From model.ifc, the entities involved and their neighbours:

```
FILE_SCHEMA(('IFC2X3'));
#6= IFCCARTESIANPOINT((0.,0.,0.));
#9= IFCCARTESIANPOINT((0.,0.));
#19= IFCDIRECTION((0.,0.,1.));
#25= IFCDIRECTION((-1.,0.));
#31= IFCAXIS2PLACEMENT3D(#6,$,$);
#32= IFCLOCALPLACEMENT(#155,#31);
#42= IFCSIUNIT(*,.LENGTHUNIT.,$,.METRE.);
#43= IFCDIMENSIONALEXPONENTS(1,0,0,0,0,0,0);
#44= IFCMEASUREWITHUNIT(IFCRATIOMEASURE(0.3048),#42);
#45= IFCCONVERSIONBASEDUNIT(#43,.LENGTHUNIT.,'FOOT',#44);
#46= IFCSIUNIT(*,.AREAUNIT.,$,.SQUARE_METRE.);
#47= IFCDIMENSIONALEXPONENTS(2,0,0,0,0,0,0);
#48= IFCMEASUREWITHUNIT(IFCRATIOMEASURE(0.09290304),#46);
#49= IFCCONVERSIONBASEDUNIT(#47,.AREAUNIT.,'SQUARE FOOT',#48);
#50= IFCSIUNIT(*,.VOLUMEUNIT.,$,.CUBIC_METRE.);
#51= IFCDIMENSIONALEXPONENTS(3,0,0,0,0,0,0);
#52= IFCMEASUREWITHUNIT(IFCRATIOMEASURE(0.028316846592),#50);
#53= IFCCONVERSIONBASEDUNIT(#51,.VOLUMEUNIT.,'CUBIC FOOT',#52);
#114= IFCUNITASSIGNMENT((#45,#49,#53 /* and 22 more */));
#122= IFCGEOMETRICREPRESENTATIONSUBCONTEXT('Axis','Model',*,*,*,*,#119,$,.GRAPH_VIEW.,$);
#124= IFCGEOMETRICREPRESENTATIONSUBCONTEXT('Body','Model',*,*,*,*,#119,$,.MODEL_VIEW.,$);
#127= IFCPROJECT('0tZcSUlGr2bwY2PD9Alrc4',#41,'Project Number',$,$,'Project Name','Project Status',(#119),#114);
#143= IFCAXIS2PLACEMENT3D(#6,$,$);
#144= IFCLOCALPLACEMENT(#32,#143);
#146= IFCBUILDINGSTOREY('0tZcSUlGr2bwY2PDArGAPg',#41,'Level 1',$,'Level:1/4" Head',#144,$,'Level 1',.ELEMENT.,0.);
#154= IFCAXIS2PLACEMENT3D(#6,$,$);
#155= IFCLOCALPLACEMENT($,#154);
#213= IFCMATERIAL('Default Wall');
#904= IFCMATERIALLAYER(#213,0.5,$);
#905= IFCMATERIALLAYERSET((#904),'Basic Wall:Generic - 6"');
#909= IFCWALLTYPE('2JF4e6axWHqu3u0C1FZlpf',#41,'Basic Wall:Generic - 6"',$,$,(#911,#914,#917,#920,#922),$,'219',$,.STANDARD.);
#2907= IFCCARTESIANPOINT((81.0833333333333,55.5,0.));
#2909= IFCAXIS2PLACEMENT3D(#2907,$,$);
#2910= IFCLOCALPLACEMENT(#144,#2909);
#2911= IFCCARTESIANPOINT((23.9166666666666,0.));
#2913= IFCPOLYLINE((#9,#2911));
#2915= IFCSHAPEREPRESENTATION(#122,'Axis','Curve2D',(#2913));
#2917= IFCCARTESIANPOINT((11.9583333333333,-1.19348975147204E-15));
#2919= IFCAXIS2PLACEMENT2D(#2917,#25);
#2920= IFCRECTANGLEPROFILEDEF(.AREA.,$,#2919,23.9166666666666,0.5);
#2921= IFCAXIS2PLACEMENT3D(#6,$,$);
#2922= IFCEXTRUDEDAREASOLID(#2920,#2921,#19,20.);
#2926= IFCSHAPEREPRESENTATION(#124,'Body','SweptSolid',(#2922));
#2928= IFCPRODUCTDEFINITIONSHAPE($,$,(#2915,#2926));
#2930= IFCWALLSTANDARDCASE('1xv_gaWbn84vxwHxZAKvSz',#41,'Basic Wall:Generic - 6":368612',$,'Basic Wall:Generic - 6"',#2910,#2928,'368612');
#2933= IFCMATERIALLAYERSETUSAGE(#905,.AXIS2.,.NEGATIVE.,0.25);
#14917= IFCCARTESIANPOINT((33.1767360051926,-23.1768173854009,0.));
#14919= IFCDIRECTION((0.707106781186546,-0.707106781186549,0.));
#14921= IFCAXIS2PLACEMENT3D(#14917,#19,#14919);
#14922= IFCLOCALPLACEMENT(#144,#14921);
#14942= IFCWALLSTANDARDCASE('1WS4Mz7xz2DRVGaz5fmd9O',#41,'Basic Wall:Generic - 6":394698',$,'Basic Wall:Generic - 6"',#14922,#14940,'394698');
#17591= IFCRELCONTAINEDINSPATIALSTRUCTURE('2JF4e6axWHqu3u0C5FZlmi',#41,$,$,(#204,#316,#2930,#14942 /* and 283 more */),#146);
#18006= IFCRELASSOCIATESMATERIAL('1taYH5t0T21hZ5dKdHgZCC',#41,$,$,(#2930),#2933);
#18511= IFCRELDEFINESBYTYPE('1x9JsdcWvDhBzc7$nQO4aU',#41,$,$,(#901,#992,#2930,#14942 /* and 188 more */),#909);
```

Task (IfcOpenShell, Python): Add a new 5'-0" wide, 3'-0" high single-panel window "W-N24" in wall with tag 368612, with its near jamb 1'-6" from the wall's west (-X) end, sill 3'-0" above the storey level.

```python
import numpy as np
import ifcopenshell
import ifcopenshell.api.feature
import ifcopenshell.api.geometry
import ifcopenshell.api.root
import ifcopenshell.api.spatial
import ifcopenshell.api.type
import ifcopenshell.geom
import ifcopenshell.util.element
import ifcopenshell.util.placement
import ifcopenshell.util.representation
import ifcopenshell.util.shape
import ifcopenshell.util.unit

model = ifcopenshell.open("model.ifc")
unit_scale = ifcopenshell.util.unit.calculate_unit_scale(model)
settings = ifcopenshell.geom.settings()


def volume(element):
    """Net volume in cubic metres, openings subtracted."""
    shape = ifcopenshell.geom.create_shape(settings, element)
    return ifcopenshell.util.shape.get_volume(shape.geometry)


wall = model.by_id(2930)
storey = ifcopenshell.util.element.get_container(wall, ifc_class="IfcBuildingStorey")
context = ifcopenshell.util.representation.get_context(model, "Model", "Body", "MODEL_VIEW")
before = volume(wall)

width, height, from_end, sill = 1.524, 0.9144, 0.4572, 0.9144  # metres

# The wall runs along its own X axis, and the end named is its -X end.
wall_shape = ifcopenshell.geom.create_shape(settings, wall)
x, y, z = ifcopenshell.util.shape.get_vertices(wall_shape.geometry).T
start = x.min() + from_end
face, thickness = float(y.min()), float(y.max() - y.min())
wall_matrix = ifcopenshell.util.placement.get_local_placement(wall.ObjectPlacement)
level = ifcopenshell.util.placement.get_local_placement(storey.ObjectPlacement)[2, 3]


def in_wall(x, y):
    """Placement at x, y metres in the wall's axes, at sill height."""
    matrix = wall_matrix.copy()
    matrix[:, 3] = wall_matrix @ np.array([x / unit_scale, y / unit_scale, 0.0, 1.0])
    matrix[2, 3] = level + sill / unit_scale
    return matrix


# Opening: a box that overshoots both wall faces by 50 mm.
opening = ifcopenshell.api.root.create_entity(model, ifc_class="IfcOpeningElement")
box = ifcopenshell.api.geometry.add_wall_representation(
    model, context=context, length=width, height=height, thickness=thickness + 0.1
)
ifcopenshell.api.geometry.assign_representation(model, product=opening, representation=box)
ifcopenshell.api.geometry.edit_object_placement(model, product=opening, matrix=in_wall(start, face - 0.05), is_si=False)
ifcopenshell.api.feature.add_feature(model, feature=opening, element=wall)

window = ifcopenshell.api.root.create_entity(model, ifc_class="IfcWindow", name="W-N24")
window.OverallWidth, window.OverallHeight = width / unit_scale, height / unit_scale
body = ifcopenshell.api.geometry.add_window_representation(
    model,
    context=context,
    overall_width=window.OverallWidth,
    overall_height=window.OverallHeight,
    partition_type="SINGLE_PANEL",
)
ifcopenshell.api.geometry.assign_representation(model, product=window, representation=body)
ifcopenshell.api.spatial.assign_container(model, products=[window], relating_structure=storey)
fills = ifcopenshell.api.feature.add_filling(model, opening=opening, element=window)
fills.OwnerHistory = window.OwnerHistory  # required in IFC2X3

# IFC2X3 keeps the operation on the window style.
style = ifcopenshell.api.root.create_entity(model, ifc_class="IfcWindowStyle", name="W-N24")
style.OperationType, style.ConstructionType = "SINGLE_PANEL", "NOTDEFINED"
style.ParameterTakesPrecedence = style.Sizeable = False
ifcopenshell.api.type.assign_type(model, related_objects=[window], relating_type=style)

# Centre the window in the wall's thickness.
ifcopenshell.api.geometry.edit_object_placement(model, product=window, matrix=in_wall(start, face), is_si=False)
window_shape = ifcopenshell.geom.create_shape(settings, window)
depth = ifcopenshell.util.shape.get_vertices(window_shape.geometry)[:, 1]
offset = face + thickness / 2 - (depth.min() + depth.max()) / 2
ifcopenshell.api.geometry.edit_object_placement(model, product=window, matrix=in_wall(start, offset), is_si=False)

after = volume(wall)

print(f"wall volume {before:.3f} -> {after:.3f} m3")

model.write("model_updated.ifc")
```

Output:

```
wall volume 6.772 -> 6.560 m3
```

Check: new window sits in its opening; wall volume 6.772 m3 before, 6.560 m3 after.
